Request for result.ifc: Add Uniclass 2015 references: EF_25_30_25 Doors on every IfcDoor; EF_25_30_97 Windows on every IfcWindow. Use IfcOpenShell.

First a look at what the model holds.

```python
import ifcopenshell

model = ifcopenshell.open("result.ifc")
print(model.schema)
print("classifications:", [c.Name for c in model.by_type("IfcClassification")])
for ifc_class in ("IfcDoor", "IfcRoof", "IfcStair", "IfcWall", "IfcWindow"):
    print(ifc_class, len(model.by_type(ifc_class)))
```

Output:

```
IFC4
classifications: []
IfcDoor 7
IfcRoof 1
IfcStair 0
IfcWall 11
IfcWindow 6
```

```python
import ifcopenshell
import ifcopenshell.api.classification

model = ifcopenshell.open("result.ifc")

system = ifcopenshell.api.classification.add_classification(model, classification="Uniclass 2015")

codes = {
    "IfcDoor": ("EF_25_30_25", "Doors"),
    "IfcWindow": ("EF_25_30_97", "Windows"),
}
for ifc_class, (code, name) in codes.items():
    products = model.by_type(ifc_class)
    ifcopenshell.api.classification.add_reference(
        model, products=products, classification=system, identification=code, name=name
    )
    print(code, len(products))

model.write("result_v2.ifc")
```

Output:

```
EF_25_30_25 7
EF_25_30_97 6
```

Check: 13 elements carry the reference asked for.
